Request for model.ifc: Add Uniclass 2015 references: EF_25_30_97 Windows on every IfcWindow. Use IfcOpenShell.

First a look at what the model holds.

```python
import ifcopenshell

model = ifcopenshell.open("model.ifc")
print(model.schema)
print("classifications:", [c.Name for c in model.by_type("IfcClassification")])
for ifc_class in ("IfcDoor", "IfcRoof", "IfcStair", "IfcWall", "IfcWindow"):
    print(ifc_class, len(model.by_type(ifc_class)))
```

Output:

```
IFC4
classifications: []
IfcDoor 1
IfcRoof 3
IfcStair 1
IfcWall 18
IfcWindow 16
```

```python
import ifcopenshell
import ifcopenshell.api.classification

model = ifcopenshell.open("model.ifc")

system = ifcopenshell.api.classification.add_classification(model, classification="Uniclass 2015")

codes = {
    "IfcWindow": ("EF_25_30_97", "Windows"),
}
for ifc_class, (code, name) in codes.items():
    products = model.by_type(ifc_class)
    ifcopenshell.api.classification.add_reference(
        model, products=products, classification=system, identification=code, name=name
    )
    print(code, len(products))

model.write("model_edited.ifc")
```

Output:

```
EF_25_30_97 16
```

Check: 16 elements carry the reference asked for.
